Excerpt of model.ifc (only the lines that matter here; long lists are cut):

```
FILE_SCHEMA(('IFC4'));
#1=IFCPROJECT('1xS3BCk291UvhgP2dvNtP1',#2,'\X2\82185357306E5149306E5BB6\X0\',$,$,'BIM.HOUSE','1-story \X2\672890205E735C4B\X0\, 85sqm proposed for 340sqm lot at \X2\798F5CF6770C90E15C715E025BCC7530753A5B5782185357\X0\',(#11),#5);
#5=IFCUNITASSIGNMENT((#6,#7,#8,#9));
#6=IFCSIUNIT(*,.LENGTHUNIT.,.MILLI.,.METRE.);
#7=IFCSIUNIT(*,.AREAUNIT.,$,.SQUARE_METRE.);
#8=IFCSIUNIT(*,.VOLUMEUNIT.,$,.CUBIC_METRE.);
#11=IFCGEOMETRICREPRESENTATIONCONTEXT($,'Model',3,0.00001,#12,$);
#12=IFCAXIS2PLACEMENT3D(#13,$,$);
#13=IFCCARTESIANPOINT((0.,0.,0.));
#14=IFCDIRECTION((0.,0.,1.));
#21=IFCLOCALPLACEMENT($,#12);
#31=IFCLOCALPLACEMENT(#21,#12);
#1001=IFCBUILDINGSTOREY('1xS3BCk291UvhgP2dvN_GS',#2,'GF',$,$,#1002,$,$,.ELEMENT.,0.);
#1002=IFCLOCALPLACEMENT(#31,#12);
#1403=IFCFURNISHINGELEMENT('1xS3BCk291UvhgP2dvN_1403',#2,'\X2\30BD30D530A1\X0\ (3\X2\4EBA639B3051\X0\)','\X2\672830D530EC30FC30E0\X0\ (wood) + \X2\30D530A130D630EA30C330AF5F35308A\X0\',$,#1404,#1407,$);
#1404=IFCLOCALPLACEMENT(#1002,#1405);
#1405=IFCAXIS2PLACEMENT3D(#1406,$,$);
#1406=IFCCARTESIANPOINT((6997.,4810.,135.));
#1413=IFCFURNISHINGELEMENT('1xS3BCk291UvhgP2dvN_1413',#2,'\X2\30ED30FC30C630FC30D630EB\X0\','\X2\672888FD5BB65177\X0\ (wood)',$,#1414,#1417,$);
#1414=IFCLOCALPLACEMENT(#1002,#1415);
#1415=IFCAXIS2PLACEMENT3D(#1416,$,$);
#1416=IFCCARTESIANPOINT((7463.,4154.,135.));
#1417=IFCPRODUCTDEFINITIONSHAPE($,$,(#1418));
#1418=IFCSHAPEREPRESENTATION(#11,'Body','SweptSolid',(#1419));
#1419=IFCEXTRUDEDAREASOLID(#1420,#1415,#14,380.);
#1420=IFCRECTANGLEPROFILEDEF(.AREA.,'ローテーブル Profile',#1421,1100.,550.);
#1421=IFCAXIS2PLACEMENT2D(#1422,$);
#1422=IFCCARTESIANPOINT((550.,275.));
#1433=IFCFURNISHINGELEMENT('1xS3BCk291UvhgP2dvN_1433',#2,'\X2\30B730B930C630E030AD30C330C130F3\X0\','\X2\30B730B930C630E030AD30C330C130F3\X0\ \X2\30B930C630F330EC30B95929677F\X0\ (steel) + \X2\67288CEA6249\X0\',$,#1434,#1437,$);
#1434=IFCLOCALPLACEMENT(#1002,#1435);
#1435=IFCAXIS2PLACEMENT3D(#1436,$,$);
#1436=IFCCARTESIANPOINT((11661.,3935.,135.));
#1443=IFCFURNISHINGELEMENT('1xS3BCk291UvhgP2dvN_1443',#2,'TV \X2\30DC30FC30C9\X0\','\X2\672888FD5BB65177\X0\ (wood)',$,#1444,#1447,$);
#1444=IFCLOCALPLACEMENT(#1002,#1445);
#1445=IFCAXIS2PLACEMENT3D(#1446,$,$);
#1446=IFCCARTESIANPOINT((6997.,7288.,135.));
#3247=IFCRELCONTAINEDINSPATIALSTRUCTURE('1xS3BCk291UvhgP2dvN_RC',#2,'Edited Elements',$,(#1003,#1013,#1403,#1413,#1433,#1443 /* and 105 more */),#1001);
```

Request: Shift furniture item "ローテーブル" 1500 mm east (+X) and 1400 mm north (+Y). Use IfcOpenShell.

```python
import ifcopenshell
import ifcopenshell.api.geometry
import ifcopenshell.util.placement
import ifcopenshell.util.unit

model = ifcopenshell.open("model.ifc")
unit_scale = ifcopenshell.util.unit.calculate_unit_scale(model)

item = model.by_guid("1xS3BCk291UvhgP2dvN_1413")
matrix = ifcopenshell.util.placement.get_local_placement(item.ObjectPlacement)
matrix[0, 3] += 1.5 / unit_scale
matrix[1, 3] += 1.4 / unit_scale
ifcopenshell.api.geometry.edit_object_placement(model, product=item, matrix=matrix, is_si=False)

print(ifcopenshell.util.placement.get_local_placement(item.ObjectPlacement).round(3) + 0.0)

model.write("model_v2.ifc")
```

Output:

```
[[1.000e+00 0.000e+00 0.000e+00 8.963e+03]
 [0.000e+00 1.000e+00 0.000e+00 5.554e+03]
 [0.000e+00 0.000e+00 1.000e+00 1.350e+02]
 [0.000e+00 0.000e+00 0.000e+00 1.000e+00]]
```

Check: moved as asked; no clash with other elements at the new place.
